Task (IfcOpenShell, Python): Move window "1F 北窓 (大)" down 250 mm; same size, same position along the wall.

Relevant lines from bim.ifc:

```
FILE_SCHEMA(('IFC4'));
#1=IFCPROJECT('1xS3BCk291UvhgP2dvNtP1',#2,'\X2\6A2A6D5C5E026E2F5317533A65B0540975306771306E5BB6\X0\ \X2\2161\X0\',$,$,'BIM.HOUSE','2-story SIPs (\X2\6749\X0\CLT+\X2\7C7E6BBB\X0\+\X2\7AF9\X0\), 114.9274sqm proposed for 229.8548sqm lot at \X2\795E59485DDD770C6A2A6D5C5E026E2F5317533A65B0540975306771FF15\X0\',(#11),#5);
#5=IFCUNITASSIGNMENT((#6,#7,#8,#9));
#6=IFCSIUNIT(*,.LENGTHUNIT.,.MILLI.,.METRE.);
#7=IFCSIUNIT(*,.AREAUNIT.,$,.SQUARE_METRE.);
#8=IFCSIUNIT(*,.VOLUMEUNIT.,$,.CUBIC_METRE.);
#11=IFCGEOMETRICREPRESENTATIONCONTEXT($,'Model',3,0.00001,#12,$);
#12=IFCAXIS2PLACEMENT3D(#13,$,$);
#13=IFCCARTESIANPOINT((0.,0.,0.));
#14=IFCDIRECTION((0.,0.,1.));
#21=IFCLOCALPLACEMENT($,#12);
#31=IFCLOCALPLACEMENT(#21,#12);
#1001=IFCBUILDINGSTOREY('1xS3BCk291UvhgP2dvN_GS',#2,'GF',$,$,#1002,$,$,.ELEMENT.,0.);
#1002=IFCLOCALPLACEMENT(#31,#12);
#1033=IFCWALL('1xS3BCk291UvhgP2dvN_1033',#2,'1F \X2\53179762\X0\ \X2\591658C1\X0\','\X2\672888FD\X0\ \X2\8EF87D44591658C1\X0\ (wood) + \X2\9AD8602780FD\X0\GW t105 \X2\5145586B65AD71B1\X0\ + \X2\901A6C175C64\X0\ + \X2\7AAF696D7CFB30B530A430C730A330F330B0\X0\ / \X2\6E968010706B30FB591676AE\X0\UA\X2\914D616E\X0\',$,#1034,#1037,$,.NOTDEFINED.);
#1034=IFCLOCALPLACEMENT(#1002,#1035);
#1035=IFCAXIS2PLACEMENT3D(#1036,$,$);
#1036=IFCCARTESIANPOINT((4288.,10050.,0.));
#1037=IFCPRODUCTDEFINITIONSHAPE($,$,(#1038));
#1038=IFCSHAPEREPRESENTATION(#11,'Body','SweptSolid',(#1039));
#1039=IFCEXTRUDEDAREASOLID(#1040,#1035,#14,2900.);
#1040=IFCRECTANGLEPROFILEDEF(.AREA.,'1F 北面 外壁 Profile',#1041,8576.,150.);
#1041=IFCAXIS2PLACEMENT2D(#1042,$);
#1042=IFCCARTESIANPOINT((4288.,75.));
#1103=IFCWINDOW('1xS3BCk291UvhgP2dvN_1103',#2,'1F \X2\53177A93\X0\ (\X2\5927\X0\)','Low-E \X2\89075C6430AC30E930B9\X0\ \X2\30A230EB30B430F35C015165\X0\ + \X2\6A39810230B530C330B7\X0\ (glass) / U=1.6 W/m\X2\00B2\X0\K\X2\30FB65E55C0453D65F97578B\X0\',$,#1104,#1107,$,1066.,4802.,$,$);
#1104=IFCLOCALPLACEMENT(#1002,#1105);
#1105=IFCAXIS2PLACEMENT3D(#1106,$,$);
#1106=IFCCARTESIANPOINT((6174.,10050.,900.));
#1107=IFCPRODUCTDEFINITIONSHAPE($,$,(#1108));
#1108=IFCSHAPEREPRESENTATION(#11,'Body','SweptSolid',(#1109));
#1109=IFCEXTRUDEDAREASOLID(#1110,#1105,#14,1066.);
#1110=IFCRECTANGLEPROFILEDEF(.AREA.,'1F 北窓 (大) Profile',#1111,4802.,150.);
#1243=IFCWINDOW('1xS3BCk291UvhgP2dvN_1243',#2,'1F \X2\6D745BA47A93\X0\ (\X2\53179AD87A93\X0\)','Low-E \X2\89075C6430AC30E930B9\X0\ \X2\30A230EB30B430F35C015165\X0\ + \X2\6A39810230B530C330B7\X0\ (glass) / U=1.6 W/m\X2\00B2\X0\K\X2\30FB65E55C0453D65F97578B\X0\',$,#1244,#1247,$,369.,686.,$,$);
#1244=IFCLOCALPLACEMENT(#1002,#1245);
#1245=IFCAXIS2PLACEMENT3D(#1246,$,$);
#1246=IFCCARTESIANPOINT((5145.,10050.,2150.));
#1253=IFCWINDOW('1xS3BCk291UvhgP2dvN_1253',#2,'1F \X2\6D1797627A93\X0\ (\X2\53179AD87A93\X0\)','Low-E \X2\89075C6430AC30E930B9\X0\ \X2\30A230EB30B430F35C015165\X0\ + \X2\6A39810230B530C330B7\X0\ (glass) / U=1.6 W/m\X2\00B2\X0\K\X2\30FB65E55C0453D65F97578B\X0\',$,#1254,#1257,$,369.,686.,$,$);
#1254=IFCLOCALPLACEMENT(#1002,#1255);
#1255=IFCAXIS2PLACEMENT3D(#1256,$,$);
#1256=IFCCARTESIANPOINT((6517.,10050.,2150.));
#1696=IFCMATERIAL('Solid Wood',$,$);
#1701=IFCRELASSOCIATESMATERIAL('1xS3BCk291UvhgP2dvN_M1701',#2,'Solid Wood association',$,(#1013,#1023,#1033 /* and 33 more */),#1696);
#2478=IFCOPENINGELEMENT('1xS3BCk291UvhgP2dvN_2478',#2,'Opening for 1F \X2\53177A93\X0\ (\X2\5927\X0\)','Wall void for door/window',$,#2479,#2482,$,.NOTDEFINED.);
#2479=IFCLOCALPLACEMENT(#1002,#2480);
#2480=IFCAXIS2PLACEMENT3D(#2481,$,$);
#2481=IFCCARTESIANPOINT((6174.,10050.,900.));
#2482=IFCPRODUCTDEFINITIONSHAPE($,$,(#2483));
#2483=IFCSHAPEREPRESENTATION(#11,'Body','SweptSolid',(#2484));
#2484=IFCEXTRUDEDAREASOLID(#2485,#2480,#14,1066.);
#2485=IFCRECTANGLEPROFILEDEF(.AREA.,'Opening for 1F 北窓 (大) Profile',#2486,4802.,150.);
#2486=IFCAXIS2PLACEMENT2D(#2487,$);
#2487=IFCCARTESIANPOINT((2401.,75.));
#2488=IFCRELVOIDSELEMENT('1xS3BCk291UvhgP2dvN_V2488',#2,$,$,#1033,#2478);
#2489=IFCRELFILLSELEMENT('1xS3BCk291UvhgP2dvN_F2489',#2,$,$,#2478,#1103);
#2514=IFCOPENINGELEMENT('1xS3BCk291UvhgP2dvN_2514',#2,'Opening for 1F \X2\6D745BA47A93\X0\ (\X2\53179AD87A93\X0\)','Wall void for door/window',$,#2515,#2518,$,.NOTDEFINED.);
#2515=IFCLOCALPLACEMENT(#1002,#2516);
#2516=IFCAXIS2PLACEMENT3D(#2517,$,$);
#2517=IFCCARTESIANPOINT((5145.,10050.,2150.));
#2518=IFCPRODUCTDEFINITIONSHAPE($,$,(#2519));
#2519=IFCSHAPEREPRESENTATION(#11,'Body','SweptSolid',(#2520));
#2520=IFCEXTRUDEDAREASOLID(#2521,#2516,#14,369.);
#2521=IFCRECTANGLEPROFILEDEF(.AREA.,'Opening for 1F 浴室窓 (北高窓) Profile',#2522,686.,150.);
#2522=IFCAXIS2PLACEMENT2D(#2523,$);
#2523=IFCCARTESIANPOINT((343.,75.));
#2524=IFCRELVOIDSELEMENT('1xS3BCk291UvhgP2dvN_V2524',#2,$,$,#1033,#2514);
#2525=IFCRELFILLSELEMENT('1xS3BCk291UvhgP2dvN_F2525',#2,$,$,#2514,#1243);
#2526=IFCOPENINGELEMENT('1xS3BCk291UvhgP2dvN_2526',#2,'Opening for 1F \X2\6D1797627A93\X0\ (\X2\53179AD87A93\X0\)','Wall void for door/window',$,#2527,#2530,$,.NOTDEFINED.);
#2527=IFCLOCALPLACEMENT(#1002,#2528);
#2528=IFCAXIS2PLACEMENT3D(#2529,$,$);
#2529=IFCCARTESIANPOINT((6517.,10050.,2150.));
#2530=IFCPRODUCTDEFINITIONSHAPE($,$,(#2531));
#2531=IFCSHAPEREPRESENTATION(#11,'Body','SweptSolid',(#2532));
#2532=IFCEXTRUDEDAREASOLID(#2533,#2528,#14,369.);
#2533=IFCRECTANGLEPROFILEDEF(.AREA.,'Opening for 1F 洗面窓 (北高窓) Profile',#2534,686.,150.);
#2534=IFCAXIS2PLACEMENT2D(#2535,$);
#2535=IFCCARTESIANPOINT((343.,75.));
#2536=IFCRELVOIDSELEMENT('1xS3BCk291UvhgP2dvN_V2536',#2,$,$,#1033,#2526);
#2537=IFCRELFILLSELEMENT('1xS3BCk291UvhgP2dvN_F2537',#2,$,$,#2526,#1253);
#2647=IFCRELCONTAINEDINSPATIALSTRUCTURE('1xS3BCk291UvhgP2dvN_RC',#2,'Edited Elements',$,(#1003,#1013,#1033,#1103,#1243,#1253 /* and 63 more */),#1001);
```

```python
import numpy as np
import ifcopenshell
import ifcopenshell.api.geometry
import ifcopenshell.util.placement
import ifcopenshell.util.unit

model = ifcopenshell.open("bim.ifc")
unit_scale = ifcopenshell.util.unit.calculate_unit_scale(model)

window = model.by_guid("1xS3BCk291UvhgP2dvN_1103")
opening = window.FillsVoids[0].RelatingOpeningElement
dz = -0.25 / unit_scale

shift = np.array([0.0, 0.0, dz])
# The window is not placed relative to its opening, so move both.
for product in (opening, window):
    matrix = ifcopenshell.util.placement.get_local_placement(product.ObjectPlacement)
    matrix[:3, 3] += shift
    ifcopenshell.api.geometry.edit_object_placement(model, product=product, matrix=matrix, is_si=False)

print(f"moved by {dz * unit_scale:+.3f} m")

model.write("bim_rev.ifc")
```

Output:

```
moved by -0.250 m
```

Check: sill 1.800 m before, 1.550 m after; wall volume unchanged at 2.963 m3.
